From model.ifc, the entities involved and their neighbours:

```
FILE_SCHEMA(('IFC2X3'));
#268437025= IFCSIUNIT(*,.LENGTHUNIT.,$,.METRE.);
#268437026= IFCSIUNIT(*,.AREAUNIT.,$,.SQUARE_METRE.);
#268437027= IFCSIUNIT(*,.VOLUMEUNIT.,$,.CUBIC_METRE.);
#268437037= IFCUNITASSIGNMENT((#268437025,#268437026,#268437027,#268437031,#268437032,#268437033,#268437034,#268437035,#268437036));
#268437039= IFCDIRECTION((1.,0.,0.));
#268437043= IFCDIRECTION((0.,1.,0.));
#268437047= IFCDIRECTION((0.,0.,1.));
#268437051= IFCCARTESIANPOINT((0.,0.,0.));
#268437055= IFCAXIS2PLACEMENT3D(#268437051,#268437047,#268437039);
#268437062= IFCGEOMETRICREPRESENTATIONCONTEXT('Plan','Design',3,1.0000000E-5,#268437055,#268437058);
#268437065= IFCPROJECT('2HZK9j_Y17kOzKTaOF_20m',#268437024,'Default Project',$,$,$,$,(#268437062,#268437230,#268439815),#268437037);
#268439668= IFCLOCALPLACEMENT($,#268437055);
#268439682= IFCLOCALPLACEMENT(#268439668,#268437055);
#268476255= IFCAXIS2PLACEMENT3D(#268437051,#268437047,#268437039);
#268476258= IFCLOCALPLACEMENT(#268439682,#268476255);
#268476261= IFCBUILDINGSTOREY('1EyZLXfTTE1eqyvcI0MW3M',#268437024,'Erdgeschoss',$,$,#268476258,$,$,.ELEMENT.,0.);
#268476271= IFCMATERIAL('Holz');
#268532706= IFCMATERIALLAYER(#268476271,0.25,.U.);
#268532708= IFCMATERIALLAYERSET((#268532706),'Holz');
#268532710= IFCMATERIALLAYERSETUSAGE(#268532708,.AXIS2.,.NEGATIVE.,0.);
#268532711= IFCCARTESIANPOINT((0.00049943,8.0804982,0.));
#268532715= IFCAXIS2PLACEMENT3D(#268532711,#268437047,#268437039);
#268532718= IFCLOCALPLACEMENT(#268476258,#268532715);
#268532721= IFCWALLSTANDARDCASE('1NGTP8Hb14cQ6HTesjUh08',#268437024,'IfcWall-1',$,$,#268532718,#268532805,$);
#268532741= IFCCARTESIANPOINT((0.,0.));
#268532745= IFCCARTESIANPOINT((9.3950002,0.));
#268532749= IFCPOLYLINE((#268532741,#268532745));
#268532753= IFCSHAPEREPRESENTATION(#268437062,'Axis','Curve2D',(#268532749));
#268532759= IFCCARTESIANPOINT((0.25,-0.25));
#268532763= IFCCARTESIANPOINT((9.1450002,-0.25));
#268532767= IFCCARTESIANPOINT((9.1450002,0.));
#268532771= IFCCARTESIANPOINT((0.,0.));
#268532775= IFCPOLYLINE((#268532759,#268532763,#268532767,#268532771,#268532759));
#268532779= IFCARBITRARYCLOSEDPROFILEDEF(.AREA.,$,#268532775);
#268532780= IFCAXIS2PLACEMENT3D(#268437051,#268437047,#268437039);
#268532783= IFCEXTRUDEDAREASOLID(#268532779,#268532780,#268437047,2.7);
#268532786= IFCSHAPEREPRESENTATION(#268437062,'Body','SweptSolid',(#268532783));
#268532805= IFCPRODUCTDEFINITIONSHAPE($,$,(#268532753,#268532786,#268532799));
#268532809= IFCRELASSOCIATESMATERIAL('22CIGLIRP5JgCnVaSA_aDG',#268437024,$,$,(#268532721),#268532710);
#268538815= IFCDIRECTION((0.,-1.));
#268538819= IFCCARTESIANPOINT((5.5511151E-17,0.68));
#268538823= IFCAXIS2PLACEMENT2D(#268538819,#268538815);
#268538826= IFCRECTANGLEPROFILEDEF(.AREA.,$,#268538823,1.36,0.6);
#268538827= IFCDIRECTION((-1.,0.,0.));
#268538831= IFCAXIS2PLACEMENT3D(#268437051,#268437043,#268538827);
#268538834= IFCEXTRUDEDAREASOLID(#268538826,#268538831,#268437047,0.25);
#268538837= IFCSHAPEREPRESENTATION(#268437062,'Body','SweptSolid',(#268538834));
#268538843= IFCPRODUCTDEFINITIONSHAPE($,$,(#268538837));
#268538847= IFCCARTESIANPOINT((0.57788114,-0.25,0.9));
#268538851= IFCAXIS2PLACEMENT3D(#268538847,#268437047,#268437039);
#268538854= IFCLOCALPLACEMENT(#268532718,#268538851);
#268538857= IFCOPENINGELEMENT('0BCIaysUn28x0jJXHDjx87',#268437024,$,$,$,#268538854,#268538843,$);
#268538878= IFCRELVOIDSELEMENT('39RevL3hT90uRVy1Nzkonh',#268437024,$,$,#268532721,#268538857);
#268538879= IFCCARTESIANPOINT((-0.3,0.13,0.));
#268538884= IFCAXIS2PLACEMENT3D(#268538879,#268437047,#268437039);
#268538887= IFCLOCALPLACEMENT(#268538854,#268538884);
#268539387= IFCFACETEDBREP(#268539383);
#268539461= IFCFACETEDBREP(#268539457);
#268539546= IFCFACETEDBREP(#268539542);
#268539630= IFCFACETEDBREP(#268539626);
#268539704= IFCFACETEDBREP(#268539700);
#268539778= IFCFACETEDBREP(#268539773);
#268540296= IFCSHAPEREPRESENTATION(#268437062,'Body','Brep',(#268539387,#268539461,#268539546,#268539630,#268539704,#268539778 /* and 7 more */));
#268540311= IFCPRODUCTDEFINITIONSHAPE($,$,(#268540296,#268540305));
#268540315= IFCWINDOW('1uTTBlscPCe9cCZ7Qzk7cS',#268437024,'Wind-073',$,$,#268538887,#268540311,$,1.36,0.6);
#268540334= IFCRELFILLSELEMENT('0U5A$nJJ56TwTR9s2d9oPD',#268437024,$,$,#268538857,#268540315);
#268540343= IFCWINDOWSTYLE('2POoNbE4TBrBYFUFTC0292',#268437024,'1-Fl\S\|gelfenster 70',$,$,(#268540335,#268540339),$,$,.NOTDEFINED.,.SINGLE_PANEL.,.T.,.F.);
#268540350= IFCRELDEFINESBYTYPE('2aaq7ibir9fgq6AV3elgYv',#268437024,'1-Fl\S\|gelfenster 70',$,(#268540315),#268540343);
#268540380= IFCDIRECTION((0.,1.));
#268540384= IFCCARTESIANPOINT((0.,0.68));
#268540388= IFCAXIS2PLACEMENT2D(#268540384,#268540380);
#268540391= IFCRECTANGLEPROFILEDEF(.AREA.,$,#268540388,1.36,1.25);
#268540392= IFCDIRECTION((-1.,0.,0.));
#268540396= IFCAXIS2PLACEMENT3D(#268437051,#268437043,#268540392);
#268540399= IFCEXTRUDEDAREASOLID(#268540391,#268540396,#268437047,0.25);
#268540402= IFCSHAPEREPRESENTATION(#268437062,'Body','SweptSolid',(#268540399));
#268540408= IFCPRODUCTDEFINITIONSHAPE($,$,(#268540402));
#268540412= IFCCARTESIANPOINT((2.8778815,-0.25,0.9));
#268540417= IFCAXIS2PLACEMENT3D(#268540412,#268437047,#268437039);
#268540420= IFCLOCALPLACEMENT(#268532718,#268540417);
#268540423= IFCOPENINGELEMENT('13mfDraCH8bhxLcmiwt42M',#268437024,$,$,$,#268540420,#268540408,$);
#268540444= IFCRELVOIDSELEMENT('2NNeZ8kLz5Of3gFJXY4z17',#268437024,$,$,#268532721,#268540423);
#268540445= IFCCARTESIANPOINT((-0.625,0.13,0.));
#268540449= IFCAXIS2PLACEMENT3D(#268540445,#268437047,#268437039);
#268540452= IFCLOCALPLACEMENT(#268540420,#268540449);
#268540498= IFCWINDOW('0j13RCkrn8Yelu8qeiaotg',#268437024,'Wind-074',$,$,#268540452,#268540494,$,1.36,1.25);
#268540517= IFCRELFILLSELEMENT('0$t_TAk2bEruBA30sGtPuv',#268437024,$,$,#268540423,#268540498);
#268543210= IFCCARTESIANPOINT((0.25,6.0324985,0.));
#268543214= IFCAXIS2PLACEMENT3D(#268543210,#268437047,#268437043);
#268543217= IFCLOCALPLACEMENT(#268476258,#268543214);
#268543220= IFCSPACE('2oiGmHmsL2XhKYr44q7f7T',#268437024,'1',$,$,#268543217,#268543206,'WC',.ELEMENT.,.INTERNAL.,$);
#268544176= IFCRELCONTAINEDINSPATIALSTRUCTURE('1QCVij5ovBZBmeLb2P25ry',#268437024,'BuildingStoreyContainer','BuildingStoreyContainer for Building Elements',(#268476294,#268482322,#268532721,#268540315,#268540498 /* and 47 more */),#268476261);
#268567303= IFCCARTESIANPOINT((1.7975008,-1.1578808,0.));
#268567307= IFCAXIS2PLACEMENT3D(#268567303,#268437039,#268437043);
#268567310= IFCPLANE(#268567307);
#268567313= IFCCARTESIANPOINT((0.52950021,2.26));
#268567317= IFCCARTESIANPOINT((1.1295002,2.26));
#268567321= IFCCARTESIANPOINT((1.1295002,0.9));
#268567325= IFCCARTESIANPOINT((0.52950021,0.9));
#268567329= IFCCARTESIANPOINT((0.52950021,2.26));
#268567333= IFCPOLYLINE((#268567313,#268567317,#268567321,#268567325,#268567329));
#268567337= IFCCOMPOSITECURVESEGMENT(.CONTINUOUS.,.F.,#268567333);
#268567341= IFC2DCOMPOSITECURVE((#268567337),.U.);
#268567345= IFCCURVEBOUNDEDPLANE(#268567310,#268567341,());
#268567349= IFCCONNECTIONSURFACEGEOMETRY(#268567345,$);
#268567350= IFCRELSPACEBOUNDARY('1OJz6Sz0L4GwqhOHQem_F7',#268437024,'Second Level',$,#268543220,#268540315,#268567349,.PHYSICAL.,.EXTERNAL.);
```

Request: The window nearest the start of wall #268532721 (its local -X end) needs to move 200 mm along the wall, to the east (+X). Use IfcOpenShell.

```python
import numpy as np
import ifcopenshell
import ifcopenshell.api.geometry
import ifcopenshell.util.placement
import ifcopenshell.util.unit

model = ifcopenshell.open("model.ifc")
unit_scale = ifcopenshell.util.unit.calculate_unit_scale(model)

window = model.by_id(268540315)
opening = window.FillsVoids[0].RelatingOpeningElement
wall = opening.VoidsElements[0].RelatingBuildingElement

wall_matrix = ifcopenshell.util.placement.get_local_placement(wall.ObjectPlacement)
shift = wall_matrix[:3, 0] * 0.2 / unit_scale
before = ifcopenshell.util.placement.get_local_placement(window.ObjectPlacement)[:3, 3].copy()

# The window is placed relative to its opening, so it follows when the opening moves.
matrix = ifcopenshell.util.placement.get_local_placement(opening.ObjectPlacement)
matrix[:3, 3] += shift
ifcopenshell.api.geometry.edit_object_placement(
    model, product=opening, matrix=matrix, is_si=False, should_transform_children=True
)

# Space boundary surfaces are stored in each space's coordinates; move them too.
for rel in window.ProvidesBoundaries:
    if not rel.ConnectionGeometry:
        continue
    surface = rel.ConnectionGeometry.SurfaceOnRelatingElement.BasisSurface
    space_matrix = ifcopenshell.util.placement.get_local_placement(rel.RelatingSpace.ObjectPlacement)
    point = np.array(surface.Position.Location.Coordinates) + space_matrix[:3, :3].T @ shift
    surface.Position = model.createIfcAxis2Placement3D(
        model.createIfcCartesianPoint(point.tolist()), surface.Position.Axis, surface.Position.RefDirection
    )

after = ifcopenshell.util.placement.get_local_placement(window.ObjectPlacement)[:3, 3]
print("window moved by", (after - before).round(3) + 0.0)

model.write("model_v2.ifc")
```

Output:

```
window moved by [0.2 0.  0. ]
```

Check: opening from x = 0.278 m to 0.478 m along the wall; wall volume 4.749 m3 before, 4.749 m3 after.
